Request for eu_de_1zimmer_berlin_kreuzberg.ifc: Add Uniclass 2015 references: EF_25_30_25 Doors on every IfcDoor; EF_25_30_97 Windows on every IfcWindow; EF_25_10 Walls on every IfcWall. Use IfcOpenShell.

First a look at what the model holds.

```python
import ifcopenshell

model = ifcopenshell.open("eu_de_1zimmer_berlin_kreuzberg.ifc")
print(model.schema)
print("classifications:", [c.Name for c in model.by_type("IfcClassification")])
for ifc_class in ("IfcDoor", "IfcRoof", "IfcStair", "IfcWall", "IfcWindow"):
    print(ifc_class, len(model.by_type(ifc_class)))
```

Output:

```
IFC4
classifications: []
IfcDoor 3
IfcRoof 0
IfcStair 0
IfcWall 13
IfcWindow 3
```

```python
import ifcopenshell
import ifcopenshell.api.classification

model = ifcopenshell.open("eu_de_1zimmer_berlin_kreuzberg.ifc")

system = ifcopenshell.api.classification.add_classification(model, classification="Uniclass 2015")

codes = {
    "IfcDoor": ("EF_25_30_25", "Doors"),
    "IfcWindow": ("EF_25_30_97", "Windows"),
    "IfcWall": ("EF_25_10", "Walls"),
}
for ifc_class, (code, name) in codes.items():
    products = model.by_type(ifc_class)
    ifcopenshell.api.classification.add_reference(
        model, products=products, classification=system, identification=code, name=name
    )
    print(code, len(products))

model.write("eu_de_1zimmer_berlin_kreuzberg-out.ifc")
```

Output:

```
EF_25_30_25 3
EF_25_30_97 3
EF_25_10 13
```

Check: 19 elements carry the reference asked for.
